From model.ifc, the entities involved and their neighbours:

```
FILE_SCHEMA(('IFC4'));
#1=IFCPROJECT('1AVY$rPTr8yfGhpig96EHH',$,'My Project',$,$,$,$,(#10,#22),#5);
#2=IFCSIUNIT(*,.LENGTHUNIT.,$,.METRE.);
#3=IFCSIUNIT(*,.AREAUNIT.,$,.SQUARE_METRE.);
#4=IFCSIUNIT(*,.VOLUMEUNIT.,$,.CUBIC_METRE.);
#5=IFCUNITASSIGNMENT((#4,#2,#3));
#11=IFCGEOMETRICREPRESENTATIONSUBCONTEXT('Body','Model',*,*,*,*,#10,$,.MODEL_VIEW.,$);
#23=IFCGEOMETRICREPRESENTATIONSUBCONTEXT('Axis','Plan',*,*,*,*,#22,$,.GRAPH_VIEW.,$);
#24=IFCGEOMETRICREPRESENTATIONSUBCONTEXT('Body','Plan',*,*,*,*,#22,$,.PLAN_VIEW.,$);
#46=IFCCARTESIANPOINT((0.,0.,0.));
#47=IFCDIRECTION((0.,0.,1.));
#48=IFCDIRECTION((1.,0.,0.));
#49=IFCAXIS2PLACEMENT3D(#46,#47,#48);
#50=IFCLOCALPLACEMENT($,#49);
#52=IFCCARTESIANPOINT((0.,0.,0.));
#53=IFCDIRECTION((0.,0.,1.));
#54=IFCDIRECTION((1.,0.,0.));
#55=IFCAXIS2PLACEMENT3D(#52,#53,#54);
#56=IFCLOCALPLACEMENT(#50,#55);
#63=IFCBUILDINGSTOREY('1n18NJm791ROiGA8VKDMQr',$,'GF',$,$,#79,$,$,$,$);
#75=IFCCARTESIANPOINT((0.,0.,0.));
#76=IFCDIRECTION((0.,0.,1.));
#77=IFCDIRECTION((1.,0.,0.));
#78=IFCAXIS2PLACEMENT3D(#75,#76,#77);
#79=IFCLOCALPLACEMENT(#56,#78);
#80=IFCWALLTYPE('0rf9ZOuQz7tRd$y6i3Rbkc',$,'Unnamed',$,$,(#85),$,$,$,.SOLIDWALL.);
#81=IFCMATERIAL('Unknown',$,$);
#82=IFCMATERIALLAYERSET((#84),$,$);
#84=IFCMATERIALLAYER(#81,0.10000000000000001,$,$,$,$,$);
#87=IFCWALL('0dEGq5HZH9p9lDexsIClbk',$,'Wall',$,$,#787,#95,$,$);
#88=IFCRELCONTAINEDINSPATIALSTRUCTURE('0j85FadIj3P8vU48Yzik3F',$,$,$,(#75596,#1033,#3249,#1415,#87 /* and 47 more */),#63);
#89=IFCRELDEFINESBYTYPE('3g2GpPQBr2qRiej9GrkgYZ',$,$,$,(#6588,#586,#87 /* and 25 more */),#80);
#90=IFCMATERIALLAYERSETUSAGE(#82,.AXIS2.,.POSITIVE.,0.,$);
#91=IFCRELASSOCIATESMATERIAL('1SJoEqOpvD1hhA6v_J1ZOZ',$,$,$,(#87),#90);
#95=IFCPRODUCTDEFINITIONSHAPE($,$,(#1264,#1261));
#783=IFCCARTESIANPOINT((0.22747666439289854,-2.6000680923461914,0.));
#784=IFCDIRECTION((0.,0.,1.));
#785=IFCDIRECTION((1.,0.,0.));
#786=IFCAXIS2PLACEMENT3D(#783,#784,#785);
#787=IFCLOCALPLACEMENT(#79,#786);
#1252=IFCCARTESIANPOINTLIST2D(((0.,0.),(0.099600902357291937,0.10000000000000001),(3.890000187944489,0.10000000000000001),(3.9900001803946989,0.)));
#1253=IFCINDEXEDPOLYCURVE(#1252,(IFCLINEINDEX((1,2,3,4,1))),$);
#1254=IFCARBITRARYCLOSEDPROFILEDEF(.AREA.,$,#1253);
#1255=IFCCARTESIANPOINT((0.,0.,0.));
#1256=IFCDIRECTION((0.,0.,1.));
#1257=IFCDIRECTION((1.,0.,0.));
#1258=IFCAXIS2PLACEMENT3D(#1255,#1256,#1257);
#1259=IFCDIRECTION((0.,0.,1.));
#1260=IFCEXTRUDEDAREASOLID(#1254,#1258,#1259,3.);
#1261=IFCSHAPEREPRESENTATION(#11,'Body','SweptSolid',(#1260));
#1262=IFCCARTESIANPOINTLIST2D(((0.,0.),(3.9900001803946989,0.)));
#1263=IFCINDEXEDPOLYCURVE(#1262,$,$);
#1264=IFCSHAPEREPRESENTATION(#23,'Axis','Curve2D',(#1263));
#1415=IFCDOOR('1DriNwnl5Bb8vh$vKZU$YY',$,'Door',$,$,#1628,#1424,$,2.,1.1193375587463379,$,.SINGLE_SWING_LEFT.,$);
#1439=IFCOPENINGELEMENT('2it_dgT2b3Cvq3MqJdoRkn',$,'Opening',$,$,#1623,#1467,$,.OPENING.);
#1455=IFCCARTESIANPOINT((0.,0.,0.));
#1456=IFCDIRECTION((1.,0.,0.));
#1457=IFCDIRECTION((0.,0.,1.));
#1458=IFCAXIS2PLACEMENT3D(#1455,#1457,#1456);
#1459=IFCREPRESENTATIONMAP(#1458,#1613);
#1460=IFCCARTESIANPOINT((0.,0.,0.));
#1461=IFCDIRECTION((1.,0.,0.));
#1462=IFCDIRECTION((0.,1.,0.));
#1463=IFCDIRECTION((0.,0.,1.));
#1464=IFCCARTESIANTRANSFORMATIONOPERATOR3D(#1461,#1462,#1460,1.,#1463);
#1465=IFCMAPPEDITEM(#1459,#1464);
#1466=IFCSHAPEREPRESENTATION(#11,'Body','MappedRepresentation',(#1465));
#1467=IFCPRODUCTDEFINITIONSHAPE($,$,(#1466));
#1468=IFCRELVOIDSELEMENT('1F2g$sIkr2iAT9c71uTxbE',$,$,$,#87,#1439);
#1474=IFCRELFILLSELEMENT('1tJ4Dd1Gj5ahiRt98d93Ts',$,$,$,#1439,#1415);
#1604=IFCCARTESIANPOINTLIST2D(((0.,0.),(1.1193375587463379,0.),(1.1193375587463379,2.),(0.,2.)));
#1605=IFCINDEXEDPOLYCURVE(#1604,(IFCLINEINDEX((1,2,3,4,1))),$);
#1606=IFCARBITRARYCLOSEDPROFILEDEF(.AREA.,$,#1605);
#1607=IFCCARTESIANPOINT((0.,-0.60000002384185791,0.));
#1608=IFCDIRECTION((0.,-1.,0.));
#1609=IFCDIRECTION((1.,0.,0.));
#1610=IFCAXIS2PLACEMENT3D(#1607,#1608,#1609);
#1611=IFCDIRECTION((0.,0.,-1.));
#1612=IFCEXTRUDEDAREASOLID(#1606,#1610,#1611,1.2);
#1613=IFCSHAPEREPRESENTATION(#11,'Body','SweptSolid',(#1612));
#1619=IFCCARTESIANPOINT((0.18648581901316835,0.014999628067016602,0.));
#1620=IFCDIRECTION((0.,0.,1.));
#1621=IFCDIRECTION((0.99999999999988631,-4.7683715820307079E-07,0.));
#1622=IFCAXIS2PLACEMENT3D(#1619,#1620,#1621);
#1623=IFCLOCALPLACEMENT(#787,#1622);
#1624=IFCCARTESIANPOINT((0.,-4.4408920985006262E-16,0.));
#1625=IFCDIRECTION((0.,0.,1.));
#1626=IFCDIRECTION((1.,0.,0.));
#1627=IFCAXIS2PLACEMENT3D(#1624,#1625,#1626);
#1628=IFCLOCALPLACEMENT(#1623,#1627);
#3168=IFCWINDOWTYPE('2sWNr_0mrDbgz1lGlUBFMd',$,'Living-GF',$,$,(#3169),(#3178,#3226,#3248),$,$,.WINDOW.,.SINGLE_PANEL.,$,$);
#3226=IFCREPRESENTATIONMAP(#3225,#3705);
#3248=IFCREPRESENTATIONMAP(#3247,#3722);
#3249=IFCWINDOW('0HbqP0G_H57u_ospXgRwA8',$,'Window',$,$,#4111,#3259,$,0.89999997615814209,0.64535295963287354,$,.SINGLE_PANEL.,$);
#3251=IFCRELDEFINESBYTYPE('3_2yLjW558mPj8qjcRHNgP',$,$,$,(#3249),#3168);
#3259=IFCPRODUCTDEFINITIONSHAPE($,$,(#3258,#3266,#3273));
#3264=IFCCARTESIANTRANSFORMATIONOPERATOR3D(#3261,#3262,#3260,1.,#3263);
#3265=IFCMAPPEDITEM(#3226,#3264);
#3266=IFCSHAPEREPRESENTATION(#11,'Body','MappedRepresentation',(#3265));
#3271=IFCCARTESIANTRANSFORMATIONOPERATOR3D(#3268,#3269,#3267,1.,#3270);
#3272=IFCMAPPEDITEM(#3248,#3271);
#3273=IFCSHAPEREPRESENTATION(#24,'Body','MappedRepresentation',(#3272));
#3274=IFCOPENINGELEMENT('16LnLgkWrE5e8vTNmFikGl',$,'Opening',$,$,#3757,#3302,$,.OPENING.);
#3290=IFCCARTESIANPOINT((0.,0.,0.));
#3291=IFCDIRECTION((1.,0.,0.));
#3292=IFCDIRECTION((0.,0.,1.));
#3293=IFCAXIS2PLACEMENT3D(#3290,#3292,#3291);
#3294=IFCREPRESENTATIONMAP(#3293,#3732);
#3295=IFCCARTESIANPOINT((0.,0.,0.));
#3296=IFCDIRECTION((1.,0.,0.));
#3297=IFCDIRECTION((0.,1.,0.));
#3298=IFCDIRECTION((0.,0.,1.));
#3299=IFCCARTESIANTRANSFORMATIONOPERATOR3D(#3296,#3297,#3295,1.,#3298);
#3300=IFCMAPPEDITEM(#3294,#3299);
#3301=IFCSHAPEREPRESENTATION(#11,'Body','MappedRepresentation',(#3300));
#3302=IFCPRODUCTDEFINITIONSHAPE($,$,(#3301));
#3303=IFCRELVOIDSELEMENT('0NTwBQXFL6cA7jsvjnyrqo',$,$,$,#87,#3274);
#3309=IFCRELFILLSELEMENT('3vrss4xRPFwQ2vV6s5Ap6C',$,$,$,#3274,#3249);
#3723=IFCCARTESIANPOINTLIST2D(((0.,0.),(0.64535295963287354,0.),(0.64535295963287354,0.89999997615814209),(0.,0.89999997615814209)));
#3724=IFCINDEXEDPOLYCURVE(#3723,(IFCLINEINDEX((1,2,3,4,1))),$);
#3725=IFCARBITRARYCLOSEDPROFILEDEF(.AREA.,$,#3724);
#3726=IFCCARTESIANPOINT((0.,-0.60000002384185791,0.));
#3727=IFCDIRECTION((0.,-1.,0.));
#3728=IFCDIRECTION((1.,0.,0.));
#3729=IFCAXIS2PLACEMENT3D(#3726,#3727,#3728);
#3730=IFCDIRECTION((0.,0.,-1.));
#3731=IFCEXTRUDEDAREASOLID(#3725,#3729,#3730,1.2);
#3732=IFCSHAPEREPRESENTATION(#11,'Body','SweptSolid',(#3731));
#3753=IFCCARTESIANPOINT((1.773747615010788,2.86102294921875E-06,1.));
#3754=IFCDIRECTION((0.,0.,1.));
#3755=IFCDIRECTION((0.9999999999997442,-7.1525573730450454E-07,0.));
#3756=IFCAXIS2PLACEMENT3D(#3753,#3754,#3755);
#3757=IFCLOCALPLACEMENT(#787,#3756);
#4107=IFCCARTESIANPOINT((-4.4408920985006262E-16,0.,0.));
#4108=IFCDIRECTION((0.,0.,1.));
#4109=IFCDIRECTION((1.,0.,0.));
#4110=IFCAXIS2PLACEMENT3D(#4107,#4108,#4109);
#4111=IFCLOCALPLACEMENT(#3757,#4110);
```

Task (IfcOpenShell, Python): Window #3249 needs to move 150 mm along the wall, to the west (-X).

```python
import ifcopenshell
import ifcopenshell.api.geometry
import ifcopenshell.util.placement

model = ifcopenshell.open("model.ifc")

window = model.by_id(3249)
opening = window.FillsVoids[0].RelatingOpeningElement
wall = opening.VoidsElements[0].RelatingBuildingElement

wall_matrix = ifcopenshell.util.placement.get_local_placement(wall.ObjectPlacement)
shift = wall_matrix[:3, 0] * -0.15
before = ifcopenshell.util.placement.get_local_placement(window.ObjectPlacement)[:3, 3].copy()

# The window is placed relative to its opening, so it follows when the opening moves.
matrix = ifcopenshell.util.placement.get_local_placement(opening.ObjectPlacement)
matrix[:3, 3] += shift
ifcopenshell.api.geometry.edit_object_placement(
    model, product=opening, matrix=matrix, is_si=False, should_transform_children=True
)

after = ifcopenshell.util.placement.get_local_placement(window.ObjectPlacement)[:3, 3]
print("window moved by", (after - before).round(3) + 0.0)

model.write("model_v2.ifc")
```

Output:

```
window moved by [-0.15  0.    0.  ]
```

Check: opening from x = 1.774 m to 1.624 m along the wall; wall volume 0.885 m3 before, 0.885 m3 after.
